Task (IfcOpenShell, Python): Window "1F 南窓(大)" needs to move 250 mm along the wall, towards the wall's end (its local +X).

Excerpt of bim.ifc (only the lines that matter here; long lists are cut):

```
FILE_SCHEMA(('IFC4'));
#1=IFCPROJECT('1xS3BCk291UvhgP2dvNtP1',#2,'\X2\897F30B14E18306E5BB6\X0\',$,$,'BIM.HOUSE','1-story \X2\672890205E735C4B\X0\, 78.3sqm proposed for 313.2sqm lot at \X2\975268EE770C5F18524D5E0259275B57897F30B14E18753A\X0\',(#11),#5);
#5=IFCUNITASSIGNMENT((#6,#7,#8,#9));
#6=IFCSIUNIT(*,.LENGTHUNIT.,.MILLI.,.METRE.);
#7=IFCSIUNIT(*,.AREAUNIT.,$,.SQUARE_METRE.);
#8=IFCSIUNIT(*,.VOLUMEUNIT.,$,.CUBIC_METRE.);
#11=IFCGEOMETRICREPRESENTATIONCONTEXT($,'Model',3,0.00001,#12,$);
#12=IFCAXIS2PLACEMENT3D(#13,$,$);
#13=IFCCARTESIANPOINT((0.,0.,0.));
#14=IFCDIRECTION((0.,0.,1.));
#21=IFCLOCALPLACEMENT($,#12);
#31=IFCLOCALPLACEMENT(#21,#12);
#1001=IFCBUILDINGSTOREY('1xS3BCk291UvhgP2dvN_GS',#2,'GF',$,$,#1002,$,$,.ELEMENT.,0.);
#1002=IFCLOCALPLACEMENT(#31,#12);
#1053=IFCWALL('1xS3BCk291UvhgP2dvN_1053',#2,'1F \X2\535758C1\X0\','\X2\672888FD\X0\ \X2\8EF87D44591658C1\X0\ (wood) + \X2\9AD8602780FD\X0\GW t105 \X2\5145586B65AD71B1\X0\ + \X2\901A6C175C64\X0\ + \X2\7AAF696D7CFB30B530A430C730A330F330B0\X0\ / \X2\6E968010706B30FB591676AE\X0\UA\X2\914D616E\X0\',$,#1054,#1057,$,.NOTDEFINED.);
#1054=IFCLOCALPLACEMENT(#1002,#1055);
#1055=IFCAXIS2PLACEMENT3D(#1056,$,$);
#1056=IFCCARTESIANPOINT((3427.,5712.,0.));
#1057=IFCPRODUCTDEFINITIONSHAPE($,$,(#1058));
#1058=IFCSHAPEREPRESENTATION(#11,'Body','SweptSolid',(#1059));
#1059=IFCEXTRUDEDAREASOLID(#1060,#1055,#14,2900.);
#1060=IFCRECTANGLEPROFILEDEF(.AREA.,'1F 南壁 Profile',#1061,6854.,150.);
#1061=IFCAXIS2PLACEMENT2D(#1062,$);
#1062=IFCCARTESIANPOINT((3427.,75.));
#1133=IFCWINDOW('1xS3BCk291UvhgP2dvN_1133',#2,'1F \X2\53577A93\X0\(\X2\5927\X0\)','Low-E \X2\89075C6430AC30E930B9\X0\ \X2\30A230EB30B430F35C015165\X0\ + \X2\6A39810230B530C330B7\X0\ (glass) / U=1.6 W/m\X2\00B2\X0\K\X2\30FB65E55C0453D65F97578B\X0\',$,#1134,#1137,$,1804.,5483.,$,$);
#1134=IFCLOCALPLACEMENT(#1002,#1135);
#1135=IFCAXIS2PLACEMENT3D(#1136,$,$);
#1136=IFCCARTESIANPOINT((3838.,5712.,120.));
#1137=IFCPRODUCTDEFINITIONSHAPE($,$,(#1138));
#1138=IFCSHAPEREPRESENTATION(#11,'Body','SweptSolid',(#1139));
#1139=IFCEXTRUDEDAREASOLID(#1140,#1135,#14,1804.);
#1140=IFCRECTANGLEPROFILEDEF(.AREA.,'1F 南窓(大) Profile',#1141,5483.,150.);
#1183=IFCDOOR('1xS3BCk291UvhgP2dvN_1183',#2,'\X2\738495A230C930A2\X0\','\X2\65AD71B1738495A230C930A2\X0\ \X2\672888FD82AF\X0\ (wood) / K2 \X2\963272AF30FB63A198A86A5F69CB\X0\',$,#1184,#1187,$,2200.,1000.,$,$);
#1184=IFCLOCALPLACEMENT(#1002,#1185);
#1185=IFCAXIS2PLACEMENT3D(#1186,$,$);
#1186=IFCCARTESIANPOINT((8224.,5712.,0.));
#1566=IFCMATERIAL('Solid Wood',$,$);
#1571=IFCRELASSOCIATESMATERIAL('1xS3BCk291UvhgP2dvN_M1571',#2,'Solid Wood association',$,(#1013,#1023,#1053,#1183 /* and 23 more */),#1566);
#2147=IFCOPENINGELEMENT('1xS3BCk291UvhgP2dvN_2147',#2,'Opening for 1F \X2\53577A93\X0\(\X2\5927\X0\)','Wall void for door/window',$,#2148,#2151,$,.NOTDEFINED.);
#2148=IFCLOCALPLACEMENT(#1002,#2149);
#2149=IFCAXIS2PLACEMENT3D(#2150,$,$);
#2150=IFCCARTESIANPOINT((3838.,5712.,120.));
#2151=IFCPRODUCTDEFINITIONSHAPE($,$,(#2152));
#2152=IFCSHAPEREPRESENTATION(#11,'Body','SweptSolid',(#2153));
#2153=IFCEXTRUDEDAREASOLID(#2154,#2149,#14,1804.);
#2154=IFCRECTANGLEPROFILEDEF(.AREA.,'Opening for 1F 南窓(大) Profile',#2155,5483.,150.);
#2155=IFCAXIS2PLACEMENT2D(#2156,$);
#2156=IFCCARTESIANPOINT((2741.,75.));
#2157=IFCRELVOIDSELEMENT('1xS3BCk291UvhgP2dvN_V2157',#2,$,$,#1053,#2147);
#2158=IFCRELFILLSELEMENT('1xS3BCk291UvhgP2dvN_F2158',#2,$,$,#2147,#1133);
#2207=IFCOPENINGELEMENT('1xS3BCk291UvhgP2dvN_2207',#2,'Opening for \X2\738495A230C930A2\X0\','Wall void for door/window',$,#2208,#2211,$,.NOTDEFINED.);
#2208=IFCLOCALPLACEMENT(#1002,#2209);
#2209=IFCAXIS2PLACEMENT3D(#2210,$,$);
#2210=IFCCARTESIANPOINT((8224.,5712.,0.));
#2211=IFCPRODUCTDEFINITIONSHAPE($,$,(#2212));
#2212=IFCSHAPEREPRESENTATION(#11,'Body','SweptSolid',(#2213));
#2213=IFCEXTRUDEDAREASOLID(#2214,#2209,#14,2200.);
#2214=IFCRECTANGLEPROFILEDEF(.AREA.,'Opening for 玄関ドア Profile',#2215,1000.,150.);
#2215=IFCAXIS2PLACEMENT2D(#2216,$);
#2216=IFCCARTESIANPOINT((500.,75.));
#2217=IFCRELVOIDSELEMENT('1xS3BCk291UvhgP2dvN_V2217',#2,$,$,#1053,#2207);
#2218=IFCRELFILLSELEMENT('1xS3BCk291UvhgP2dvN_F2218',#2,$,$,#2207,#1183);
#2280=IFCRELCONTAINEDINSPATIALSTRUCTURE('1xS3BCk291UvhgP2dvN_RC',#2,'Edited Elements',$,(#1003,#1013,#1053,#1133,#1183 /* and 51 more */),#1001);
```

```python
import ifcopenshell
import ifcopenshell.api.geometry
import ifcopenshell.util.placement
import ifcopenshell.util.unit

model = ifcopenshell.open("bim.ifc")
unit_scale = ifcopenshell.util.unit.calculate_unit_scale(model)

window = model.by_id(1133)
opening = window.FillsVoids[0].RelatingOpeningElement
wall = opening.VoidsElements[0].RelatingBuildingElement

wall_matrix = ifcopenshell.util.placement.get_local_placement(wall.ObjectPlacement)
shift = wall_matrix[:3, 0] * 0.25 / unit_scale
before = ifcopenshell.util.placement.get_local_placement(window.ObjectPlacement)[:3, 3].copy()

# The window is not placed relative to its opening, so move both.
for product in (opening, window):
    matrix = ifcopenshell.util.placement.get_local_placement(product.ObjectPlacement)
    matrix[:3, 3] += shift
    ifcopenshell.api.geometry.edit_object_placement(model, product=product, matrix=matrix, is_si=False)

after = ifcopenshell.util.placement.get_local_placement(window.ObjectPlacement)[:3, 3]
print("window moved by", (after - before).round(3) + 0.0)

model.write("bim_rev.ifc")
```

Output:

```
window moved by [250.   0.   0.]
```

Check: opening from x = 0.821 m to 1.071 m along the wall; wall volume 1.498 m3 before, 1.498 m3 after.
